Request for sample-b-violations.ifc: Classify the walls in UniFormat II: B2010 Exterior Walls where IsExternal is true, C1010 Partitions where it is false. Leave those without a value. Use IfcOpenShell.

First a look at what the model holds.

```python
import ifcopenshell
import ifcopenshell.util.element

model = ifcopenshell.open("sample-b-violations.ifc")
print(model.schema)
print("classifications:", [c.Name for c in model.by_type("IfcClassification")])
values = [ifcopenshell.util.element.get_pset(e, "Pset_WallCommon", "IsExternal") for e in model.by_type("IfcWall")]
for value in (True, False, None):
    print("IsExternal", value, values.count(value))
```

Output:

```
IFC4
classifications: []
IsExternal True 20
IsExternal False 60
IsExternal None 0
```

```python
import ifcopenshell
import ifcopenshell.api.classification
import ifcopenshell.util.element

model = ifcopenshell.open("sample-b-violations.ifc")

system = ifcopenshell.api.classification.add_classification(model, classification="UniFormat II")

walls = model.by_type("IfcWall")
external = {e: ifcopenshell.util.element.get_pset(e, "Pset_WallCommon", "IsExternal") for e in walls}
for flag, code, name in ((True, "B2010", "Exterior Walls"), (False, "C1010", "Partitions")):
    products = [e for e in walls if external[e] is flag]
    ifcopenshell.api.classification.add_reference(
        model, products=products, classification=system, identification=code, name=name
    )
    print(code, len(products))

model.write("sample-b-violations_v2.ifc")
```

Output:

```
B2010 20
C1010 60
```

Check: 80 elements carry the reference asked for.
